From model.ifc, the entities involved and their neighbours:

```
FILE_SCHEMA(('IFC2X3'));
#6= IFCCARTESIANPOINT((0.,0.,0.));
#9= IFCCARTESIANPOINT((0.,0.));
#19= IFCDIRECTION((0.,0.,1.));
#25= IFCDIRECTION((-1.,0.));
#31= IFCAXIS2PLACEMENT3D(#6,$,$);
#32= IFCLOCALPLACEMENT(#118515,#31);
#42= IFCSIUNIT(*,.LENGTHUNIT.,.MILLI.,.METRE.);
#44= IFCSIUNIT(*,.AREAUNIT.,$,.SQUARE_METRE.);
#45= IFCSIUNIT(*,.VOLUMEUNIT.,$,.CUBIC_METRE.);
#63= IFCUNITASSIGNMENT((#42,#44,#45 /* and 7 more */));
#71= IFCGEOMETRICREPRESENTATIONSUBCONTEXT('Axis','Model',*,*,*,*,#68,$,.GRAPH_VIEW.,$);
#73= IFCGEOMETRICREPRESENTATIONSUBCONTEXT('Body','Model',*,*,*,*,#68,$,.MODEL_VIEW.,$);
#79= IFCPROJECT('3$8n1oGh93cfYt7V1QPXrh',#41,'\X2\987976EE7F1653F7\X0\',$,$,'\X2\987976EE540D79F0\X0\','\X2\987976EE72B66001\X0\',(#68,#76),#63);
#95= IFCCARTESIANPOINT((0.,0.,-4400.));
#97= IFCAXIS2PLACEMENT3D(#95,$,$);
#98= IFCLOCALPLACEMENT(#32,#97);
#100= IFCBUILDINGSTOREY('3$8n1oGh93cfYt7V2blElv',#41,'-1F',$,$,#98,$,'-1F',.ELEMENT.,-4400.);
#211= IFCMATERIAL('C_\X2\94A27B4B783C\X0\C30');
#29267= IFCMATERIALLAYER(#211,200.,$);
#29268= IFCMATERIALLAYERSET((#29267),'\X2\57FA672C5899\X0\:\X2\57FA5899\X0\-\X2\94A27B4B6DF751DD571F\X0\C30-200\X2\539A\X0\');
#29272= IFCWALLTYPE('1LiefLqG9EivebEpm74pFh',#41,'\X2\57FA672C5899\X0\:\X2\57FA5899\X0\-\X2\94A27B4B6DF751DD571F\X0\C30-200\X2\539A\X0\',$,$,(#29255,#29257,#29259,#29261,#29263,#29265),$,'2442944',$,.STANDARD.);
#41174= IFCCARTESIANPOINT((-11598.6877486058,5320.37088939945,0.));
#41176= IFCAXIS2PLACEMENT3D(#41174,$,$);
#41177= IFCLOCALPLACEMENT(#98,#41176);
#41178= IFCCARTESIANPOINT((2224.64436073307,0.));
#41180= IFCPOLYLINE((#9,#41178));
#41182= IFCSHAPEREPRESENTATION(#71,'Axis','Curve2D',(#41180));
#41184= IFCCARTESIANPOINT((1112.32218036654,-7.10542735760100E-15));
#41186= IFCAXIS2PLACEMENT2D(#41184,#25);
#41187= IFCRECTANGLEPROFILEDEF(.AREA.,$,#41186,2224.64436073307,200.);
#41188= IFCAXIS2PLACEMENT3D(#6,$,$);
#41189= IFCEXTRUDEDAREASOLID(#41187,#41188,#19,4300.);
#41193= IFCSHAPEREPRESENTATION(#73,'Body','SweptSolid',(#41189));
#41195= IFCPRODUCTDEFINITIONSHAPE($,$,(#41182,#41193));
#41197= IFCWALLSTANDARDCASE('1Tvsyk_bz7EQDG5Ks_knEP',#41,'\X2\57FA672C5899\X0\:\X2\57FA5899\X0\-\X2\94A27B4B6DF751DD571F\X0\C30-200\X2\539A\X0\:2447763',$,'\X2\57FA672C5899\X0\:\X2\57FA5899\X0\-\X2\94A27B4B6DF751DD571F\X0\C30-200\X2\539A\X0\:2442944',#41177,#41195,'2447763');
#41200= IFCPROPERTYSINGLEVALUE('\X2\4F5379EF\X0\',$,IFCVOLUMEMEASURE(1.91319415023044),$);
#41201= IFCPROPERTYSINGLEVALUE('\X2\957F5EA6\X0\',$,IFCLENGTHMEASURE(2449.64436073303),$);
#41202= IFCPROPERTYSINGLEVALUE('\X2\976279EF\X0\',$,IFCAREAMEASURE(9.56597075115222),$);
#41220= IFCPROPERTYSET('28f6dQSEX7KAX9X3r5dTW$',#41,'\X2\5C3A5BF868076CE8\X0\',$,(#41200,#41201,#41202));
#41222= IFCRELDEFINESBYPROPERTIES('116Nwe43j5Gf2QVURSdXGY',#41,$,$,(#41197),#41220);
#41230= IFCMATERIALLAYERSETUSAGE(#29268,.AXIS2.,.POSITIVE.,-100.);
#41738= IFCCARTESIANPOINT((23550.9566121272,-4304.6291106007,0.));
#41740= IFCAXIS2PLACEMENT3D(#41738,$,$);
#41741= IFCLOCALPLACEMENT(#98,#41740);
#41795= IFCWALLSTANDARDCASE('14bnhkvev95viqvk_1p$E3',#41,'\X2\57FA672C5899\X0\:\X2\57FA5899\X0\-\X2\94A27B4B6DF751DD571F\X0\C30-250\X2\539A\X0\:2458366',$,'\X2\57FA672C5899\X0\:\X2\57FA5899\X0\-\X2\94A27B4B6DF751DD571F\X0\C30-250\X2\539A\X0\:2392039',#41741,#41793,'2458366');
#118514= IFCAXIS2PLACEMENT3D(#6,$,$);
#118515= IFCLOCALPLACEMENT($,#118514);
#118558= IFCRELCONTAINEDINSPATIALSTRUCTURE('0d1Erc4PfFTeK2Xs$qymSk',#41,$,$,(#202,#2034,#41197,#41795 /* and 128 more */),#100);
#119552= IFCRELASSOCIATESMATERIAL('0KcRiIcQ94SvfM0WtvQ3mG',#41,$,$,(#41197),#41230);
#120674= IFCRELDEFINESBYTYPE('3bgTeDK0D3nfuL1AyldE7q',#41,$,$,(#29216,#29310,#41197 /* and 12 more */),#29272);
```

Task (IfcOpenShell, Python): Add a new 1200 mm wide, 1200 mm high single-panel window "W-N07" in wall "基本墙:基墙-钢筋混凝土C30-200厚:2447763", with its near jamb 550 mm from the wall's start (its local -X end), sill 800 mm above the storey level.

```python
import numpy as np
import ifcopenshell
import ifcopenshell.api.feature
import ifcopenshell.api.geometry
import ifcopenshell.api.pset
import ifcopenshell.api.root
import ifcopenshell.api.spatial
import ifcopenshell.api.type
import ifcopenshell.geom
import ifcopenshell.util.element
import ifcopenshell.util.placement
import ifcopenshell.util.representation
import ifcopenshell.util.shape
import ifcopenshell.util.unit

model = ifcopenshell.open("model.ifc")
unit_scale = ifcopenshell.util.unit.calculate_unit_scale(model)
area_scale = ifcopenshell.util.unit.calculate_unit_scale(model, "AREAUNIT")
volume_scale = ifcopenshell.util.unit.calculate_unit_scale(model, "VOLUMEUNIT")
settings = ifcopenshell.geom.settings()


def volume(element):
    """Net volume in cubic metres, openings subtracted."""
    shape = ifcopenshell.geom.create_shape(settings, element)
    return ifcopenshell.util.shape.get_volume(shape.geometry)


wall = model.by_guid("1Tvsyk_bz7EQDG5Ks_knEP")
storey = ifcopenshell.util.element.get_container(wall, ifc_class="IfcBuildingStorey")
context = ifcopenshell.util.representation.get_context(model, "Model", "Body", "MODEL_VIEW")
before = volume(wall)

width, height, from_end, sill = 1.2, 1.2, 0.55, 0.8  # metres

# The wall runs along its own X axis, and the end named is its -X end.
wall_shape = ifcopenshell.geom.create_shape(settings, wall)
x, y, z = ifcopenshell.util.shape.get_vertices(wall_shape.geometry).T
start = x.min() + from_end
face, thickness = float(y.min()), float(y.max() - y.min())
wall_matrix = ifcopenshell.util.placement.get_local_placement(wall.ObjectPlacement)
level = ifcopenshell.util.placement.get_local_placement(storey.ObjectPlacement)[2, 3]


def in_wall(x, y):
    """Placement at x, y metres in the wall's axes, at sill height."""
    matrix = wall_matrix.copy()
    matrix[:, 3] = wall_matrix @ np.array([x / unit_scale, y / unit_scale, 0.0, 1.0])
    matrix[2, 3] = level + sill / unit_scale
    return matrix


# Opening: a box that overshoots both wall faces by 50 mm.
opening = ifcopenshell.api.root.create_entity(model, ifc_class="IfcOpeningElement")
box = ifcopenshell.api.geometry.add_wall_representation(
    model, context=context, length=width, height=height, thickness=thickness + 0.1
)
ifcopenshell.api.geometry.assign_representation(model, product=opening, representation=box)
ifcopenshell.api.geometry.edit_object_placement(model, product=opening, matrix=in_wall(start, face - 0.05), is_si=False)
ifcopenshell.api.feature.add_feature(model, feature=opening, element=wall)

window = ifcopenshell.api.root.create_entity(model, ifc_class="IfcWindow", name="W-N07")
window.OverallWidth, window.OverallHeight = width / unit_scale, height / unit_scale
body = ifcopenshell.api.geometry.add_window_representation(
    model,
    context=context,
    overall_width=window.OverallWidth,
    overall_height=window.OverallHeight,
    partition_type="SINGLE_PANEL",
)
ifcopenshell.api.geometry.assign_representation(model, product=window, representation=body)
ifcopenshell.api.spatial.assign_container(model, products=[window], relating_structure=storey)
fills = ifcopenshell.api.feature.add_filling(model, opening=opening, element=window)
fills.OwnerHistory = window.OwnerHistory  # required in IFC2X3

# IFC2X3 keeps the operation on the window style.
style = ifcopenshell.api.root.create_entity(model, ifc_class="IfcWindowStyle", name="W-N07")
style.OperationType, style.ConstructionType = "SINGLE_PANEL", "NOTDEFINED"
style.ParameterTakesPrecedence = style.Sizeable = False
ifcopenshell.api.type.assign_type(model, related_objects=[window], relating_type=style)

# Centre the window in the wall's thickness.
ifcopenshell.api.geometry.edit_object_placement(model, product=window, matrix=in_wall(start, face), is_si=False)
window_shape = ifcopenshell.geom.create_shape(settings, window)
depth = ifcopenshell.util.shape.get_vertices(window_shape.geometry)[:, 1]
offset = face + thickness / 2 - (depth.min() + depth.max()) / 2
ifcopenshell.api.geometry.edit_object_placement(model, product=window, matrix=in_wall(start, offset), is_si=False)

after = volume(wall)

# Update the wall's stored quantities.
pset = model.by_id(ifcopenshell.util.element.get_pset(wall, "尺寸标注", should_inherit=False)["id"])
ifcopenshell.api.pset.edit_pset(model, pset=pset, properties={
    "体积": model.create_entity("IfcVolumeMeasure", after / volume_scale),
    "面积": model.create_entity("IfcAreaMeasure", after / thickness / area_scale),
})

print(f"wall volume {before:.3f} -> {after:.3f} m3")

model.write("model_updated.ifc")
```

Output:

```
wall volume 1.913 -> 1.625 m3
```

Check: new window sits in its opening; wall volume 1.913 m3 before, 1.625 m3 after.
